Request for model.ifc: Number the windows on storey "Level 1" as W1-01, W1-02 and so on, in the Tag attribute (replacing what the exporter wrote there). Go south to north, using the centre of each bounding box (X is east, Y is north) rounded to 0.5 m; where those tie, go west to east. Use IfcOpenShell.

First a look at what the model holds.

```python
import ifcopenshell
import ifcopenshell.util.element
import ifcopenshell.util.placement

model = ifcopenshell.open("model.ifc")
print(model.schema)
storey = next(s for s in model.by_type("IfcBuildingStorey") if s.Name == "Level 1")
windows = [e for e in ifcopenshell.util.element.get_decomposition(storey) if e.is_a("IfcWindow")]
for e in sorted(windows, key=lambda e: e.id()):
    origin = ifcopenshell.util.placement.get_local_placement(e.ObjectPlacement)[:3, 3]
    print(e.id(), e.Tag, e.Name, origin.round(2) + 0.0, sep=" | ")
```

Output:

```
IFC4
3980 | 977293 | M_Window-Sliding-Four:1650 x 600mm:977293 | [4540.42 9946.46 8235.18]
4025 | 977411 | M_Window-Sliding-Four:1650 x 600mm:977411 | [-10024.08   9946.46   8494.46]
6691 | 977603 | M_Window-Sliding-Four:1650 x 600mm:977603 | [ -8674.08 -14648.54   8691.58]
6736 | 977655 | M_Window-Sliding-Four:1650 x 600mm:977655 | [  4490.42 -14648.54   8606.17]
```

```python
import ifcopenshell
import ifcopenshell.geom
import ifcopenshell.util.element
import ifcopenshell.util.shape

model = ifcopenshell.open("model.ifc")
settings = ifcopenshell.geom.settings()
settings.set("use-world-coords", True)


def centre(element):
    shape = ifcopenshell.geom.create_shape(settings, element)
    return ifcopenshell.util.shape.get_bbox_centroid(shape.geometry)


storey = next(s for s in model.by_type("IfcBuildingStorey") if s.Name == "Level 1")
windows = [e for e in ifcopenshell.util.element.get_decomposition(storey) if e.is_a("IfcWindow")]

# Insertion points can sit at a corner or the storey origin, so sort by the geometry (in metres).
centres = {e: centre(e) for e in windows}
windows.sort(key=lambda e: (round(centres[e][1] / 0.5), centres[e][0]))

for i, e in enumerate(windows, start=1):
    number = f"W1-{i:02d}"
    e.Tag = number
    print(e.id(), number)

model.write("model_rev.ifc")
```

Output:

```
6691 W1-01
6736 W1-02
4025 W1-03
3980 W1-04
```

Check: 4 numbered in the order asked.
